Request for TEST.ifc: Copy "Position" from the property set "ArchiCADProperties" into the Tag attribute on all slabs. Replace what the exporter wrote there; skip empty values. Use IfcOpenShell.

First a look at what the model holds.

```python
import ifcopenshell
import ifcopenshell.util.element

model = ifcopenshell.open("TEST.ifc")
print(model.schema)
slabs = model.by_type("IfcSlab")
print(len(slabs), "slabs")
for e in slabs[:8]:
    source = ifcopenshell.util.element.get_pset(e, "ArchiCADProperties", "Position")
    target = e.Tag
    print(e.id(), repr(source), repr(target), sep=" | ")
```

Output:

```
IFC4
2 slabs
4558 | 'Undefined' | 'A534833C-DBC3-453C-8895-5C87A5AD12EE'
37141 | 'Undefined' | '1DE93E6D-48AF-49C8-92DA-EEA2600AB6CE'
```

```python
import ifcopenshell
import ifcopenshell.util.element

model = ifcopenshell.open("TEST.ifc")

count = 0
for e in model.by_type("IfcSlab"):
    value = ifcopenshell.util.element.get_pset(e, "ArchiCADProperties", "Position")
    current = e.Tag
    if not value or not value.strip() or current == value:
        continue
    e.Tag = value
    count += 1

print(count, "slabs updated")

model.write("TEST-out.ifc")
```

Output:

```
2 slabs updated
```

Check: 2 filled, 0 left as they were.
